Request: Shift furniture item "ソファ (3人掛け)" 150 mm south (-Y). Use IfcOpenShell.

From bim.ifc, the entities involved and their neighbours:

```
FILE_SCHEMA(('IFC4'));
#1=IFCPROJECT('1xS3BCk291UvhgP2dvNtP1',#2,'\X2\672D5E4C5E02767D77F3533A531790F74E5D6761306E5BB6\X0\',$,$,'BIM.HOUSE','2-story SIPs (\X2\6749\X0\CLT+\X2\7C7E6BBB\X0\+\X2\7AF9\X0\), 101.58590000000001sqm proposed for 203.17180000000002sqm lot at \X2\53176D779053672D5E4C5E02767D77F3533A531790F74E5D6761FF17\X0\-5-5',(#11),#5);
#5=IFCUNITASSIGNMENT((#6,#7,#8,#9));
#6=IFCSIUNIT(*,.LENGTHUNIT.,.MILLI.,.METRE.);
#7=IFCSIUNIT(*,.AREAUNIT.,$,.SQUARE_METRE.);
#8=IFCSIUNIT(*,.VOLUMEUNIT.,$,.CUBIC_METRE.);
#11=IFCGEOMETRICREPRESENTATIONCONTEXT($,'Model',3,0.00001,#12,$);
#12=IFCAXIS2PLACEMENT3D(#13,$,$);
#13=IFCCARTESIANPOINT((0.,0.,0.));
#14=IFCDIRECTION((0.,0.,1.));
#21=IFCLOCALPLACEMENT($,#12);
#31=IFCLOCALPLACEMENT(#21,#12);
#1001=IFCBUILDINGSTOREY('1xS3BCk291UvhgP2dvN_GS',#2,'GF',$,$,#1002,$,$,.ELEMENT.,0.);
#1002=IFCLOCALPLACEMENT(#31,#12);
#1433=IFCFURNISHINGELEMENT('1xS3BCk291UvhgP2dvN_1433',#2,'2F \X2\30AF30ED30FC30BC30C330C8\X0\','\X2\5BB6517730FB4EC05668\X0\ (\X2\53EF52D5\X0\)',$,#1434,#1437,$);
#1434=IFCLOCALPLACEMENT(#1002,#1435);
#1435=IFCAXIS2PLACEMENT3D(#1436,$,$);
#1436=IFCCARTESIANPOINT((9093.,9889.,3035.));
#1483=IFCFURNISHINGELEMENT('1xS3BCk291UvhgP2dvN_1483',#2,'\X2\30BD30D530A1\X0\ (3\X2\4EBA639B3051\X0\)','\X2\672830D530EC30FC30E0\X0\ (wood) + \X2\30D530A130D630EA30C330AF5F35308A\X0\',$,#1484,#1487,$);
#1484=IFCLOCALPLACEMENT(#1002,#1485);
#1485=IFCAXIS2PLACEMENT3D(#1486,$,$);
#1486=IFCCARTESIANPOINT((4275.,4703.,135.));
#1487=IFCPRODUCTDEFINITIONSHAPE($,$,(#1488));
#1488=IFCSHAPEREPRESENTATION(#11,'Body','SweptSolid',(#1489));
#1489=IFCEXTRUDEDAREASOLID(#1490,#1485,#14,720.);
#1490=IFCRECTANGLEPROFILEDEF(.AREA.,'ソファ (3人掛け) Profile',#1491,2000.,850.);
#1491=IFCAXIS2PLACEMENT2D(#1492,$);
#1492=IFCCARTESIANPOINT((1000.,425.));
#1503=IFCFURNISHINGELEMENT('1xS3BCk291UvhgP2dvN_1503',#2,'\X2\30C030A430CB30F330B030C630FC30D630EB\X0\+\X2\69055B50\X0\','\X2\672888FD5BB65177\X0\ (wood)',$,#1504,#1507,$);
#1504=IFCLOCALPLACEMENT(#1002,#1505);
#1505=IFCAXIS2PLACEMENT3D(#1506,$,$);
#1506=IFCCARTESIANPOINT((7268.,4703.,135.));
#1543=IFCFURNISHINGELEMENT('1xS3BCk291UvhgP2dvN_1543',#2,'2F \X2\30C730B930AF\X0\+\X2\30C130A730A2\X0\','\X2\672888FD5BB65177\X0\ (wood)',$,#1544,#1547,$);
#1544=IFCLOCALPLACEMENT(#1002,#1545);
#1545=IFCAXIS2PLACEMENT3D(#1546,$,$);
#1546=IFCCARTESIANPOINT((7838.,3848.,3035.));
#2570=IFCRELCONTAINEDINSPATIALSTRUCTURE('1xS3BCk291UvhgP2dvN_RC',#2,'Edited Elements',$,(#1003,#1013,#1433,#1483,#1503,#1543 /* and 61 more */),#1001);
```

```python
import ifcopenshell
import ifcopenshell.api.geometry
import ifcopenshell.util.placement
import ifcopenshell.util.unit

model = ifcopenshell.open("bim.ifc")
unit_scale = ifcopenshell.util.unit.calculate_unit_scale(model)

item = model.by_guid("1xS3BCk291UvhgP2dvN_1483")
matrix = ifcopenshell.util.placement.get_local_placement(item.ObjectPlacement)
matrix[1, 3] -= 0.15 / unit_scale
ifcopenshell.api.geometry.edit_object_placement(model, product=item, matrix=matrix, is_si=False)

print(ifcopenshell.util.placement.get_local_placement(item.ObjectPlacement).round(3) + 0.0)

model.write("bim_edited.ifc")
```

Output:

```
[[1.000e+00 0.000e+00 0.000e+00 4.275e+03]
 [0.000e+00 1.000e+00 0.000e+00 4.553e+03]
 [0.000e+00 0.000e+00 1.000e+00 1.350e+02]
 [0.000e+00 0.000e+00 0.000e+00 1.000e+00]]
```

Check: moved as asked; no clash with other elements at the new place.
